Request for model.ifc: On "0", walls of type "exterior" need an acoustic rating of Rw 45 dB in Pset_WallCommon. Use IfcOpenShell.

First a look at what the model holds.

```python
import ifcopenshell
import ifcopenshell.util.element

model = ifcopenshell.open("model.ifc")
print(model.schema)
storey = next(s for s in model.by_type("IfcBuildingStorey") if s.Name == "0")
walls = [e for e in ifcopenshell.util.element.get_decomposition(storey) if e.is_a("IfcWall")]
seen = {}
for e in walls:
    element_type = ifcopenshell.util.element.get_type(e)
    key = (element_type.Name if element_type != e and element_type else None, ifcopenshell.util.element.get_pset(e, "Pset_WallCommon", "AcousticRating"))
    seen[key] = seen.get(key, 0) + 1
for (name, value), count in sorted(seen.items(), key=str):
    print(count, "x", name, "|", value)
```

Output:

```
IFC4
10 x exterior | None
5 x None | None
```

```python
import ifcopenshell
import ifcopenshell.api.pset
import ifcopenshell.util.element

model = ifcopenshell.open("model.ifc")

storey = next(s for s in model.by_type("IfcBuildingStorey") if s.Name == "0")
walls = [e for e in ifcopenshell.util.element.get_decomposition(storey) if e.is_a("IfcWall")]

count = 0
for e in walls:
    element_type = ifcopenshell.util.element.get_type(e)
    if element_type in (None, e) or element_type.Name != "exterior":
        continue
    # add_pset returns the element's existing set when there is one.
    pset = ifcopenshell.api.pset.add_pset(model, product=e, name="Pset_WallCommon")
    ifcopenshell.api.pset.edit_pset(model, pset=pset, properties={"AcousticRating": "Rw 45 dB"})
    count += 1

print(count, "walls updated")

model.write("model_updated.ifc")
```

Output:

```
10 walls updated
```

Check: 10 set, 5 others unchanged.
